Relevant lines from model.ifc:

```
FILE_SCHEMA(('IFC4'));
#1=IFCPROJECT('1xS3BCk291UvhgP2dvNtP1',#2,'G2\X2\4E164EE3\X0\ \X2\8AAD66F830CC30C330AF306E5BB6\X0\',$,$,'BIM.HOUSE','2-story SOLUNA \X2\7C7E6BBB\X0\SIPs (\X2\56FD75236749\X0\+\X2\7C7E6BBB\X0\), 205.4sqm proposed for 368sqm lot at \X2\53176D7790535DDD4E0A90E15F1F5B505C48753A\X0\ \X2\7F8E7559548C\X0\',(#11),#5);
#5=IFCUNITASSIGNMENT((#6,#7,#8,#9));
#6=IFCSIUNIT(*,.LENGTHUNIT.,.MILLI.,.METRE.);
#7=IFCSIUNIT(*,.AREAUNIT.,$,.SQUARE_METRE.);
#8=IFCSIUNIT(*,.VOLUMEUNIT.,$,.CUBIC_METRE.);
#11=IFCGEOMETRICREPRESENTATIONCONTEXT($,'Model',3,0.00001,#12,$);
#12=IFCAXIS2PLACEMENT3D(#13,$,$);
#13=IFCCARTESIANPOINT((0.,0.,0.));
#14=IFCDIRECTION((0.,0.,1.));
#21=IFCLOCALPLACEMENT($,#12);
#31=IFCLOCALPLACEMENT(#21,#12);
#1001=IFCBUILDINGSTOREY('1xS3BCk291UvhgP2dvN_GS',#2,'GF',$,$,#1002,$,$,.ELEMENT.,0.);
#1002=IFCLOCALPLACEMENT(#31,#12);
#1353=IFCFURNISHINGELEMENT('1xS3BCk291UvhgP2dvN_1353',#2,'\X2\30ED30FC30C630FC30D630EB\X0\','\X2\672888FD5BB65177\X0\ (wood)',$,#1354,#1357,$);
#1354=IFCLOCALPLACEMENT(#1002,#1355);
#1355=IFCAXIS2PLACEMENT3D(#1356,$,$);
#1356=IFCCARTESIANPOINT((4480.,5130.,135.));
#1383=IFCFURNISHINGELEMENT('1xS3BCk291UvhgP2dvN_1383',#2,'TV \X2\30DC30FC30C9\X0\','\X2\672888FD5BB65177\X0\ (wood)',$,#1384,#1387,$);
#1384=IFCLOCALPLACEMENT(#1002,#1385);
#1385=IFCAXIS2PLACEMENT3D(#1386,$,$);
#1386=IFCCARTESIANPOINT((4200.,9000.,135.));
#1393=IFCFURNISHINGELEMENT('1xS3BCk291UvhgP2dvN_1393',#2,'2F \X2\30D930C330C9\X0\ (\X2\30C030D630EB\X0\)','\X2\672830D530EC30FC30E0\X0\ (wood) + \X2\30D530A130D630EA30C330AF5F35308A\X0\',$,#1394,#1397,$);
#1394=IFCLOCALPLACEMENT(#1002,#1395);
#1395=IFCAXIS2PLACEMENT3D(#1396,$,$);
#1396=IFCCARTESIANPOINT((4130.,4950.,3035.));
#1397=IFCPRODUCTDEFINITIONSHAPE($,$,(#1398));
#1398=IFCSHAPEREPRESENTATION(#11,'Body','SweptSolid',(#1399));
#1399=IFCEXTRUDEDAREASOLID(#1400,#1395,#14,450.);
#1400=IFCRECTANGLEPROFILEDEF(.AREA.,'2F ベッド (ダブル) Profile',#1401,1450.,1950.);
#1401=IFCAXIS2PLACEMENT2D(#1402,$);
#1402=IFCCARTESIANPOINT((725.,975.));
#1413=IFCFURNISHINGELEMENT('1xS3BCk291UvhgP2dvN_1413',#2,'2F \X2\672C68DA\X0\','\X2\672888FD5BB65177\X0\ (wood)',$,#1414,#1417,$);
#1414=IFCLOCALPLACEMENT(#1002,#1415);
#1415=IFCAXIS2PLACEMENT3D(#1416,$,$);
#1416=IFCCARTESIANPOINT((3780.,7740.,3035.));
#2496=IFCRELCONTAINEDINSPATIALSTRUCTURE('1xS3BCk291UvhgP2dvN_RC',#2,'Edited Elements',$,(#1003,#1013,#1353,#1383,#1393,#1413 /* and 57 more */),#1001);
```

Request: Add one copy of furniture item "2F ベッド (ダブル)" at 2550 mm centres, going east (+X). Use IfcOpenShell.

```python
import numpy as np
import ifcopenshell
import ifcopenshell.api.geometry
import ifcopenshell.api.root
import ifcopenshell.util.element
import ifcopenshell.util.placement
import ifcopenshell.util.unit

model = ifcopenshell.open("model.ifc")
unit_scale = ifcopenshell.util.unit.calculate_unit_scale(model)


def reuse_history(source, copy):
    """copy_class also copies each property set's owner history, people and application; keep the originals."""
    for rel in copy.IsDefinedBy:
        if rel.is_a("IfcRelDefinesByProperties") and (history := rel.RelatingPropertyDefinition.OwnerHistory):
            rel.RelatingPropertyDefinition.OwnerHistory = source.OwnerHistory
            ifcopenshell.util.element.remove_deep2(model, history)


source = model.by_id(1393)
base = ifcopenshell.util.placement.get_local_placement(source.ObjectPlacement)
step = np.array([1.0, 0.0, 0.0]) * 2.55 / unit_scale

for i in range(1, 2):
    copy = ifcopenshell.api.root.copy_class(model, product=source)
    copy.Representation = ifcopenshell.util.element.copy_deep(
        model, source.Representation, exclude=["IfcGeometricRepresentationContext", "IfcRepresentationMap"]
    )
    reuse_history(source, copy)
    matrix = base.copy()
    matrix[:3, 3] += i * step
    print("added at", matrix[:3, 3].round(3) + 0.0)
    ifcopenshell.api.geometry.edit_object_placement(model, product=copy, matrix=matrix, is_si=False)

model.write("model_updated.ifc")
```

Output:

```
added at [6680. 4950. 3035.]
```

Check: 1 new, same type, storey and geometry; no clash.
